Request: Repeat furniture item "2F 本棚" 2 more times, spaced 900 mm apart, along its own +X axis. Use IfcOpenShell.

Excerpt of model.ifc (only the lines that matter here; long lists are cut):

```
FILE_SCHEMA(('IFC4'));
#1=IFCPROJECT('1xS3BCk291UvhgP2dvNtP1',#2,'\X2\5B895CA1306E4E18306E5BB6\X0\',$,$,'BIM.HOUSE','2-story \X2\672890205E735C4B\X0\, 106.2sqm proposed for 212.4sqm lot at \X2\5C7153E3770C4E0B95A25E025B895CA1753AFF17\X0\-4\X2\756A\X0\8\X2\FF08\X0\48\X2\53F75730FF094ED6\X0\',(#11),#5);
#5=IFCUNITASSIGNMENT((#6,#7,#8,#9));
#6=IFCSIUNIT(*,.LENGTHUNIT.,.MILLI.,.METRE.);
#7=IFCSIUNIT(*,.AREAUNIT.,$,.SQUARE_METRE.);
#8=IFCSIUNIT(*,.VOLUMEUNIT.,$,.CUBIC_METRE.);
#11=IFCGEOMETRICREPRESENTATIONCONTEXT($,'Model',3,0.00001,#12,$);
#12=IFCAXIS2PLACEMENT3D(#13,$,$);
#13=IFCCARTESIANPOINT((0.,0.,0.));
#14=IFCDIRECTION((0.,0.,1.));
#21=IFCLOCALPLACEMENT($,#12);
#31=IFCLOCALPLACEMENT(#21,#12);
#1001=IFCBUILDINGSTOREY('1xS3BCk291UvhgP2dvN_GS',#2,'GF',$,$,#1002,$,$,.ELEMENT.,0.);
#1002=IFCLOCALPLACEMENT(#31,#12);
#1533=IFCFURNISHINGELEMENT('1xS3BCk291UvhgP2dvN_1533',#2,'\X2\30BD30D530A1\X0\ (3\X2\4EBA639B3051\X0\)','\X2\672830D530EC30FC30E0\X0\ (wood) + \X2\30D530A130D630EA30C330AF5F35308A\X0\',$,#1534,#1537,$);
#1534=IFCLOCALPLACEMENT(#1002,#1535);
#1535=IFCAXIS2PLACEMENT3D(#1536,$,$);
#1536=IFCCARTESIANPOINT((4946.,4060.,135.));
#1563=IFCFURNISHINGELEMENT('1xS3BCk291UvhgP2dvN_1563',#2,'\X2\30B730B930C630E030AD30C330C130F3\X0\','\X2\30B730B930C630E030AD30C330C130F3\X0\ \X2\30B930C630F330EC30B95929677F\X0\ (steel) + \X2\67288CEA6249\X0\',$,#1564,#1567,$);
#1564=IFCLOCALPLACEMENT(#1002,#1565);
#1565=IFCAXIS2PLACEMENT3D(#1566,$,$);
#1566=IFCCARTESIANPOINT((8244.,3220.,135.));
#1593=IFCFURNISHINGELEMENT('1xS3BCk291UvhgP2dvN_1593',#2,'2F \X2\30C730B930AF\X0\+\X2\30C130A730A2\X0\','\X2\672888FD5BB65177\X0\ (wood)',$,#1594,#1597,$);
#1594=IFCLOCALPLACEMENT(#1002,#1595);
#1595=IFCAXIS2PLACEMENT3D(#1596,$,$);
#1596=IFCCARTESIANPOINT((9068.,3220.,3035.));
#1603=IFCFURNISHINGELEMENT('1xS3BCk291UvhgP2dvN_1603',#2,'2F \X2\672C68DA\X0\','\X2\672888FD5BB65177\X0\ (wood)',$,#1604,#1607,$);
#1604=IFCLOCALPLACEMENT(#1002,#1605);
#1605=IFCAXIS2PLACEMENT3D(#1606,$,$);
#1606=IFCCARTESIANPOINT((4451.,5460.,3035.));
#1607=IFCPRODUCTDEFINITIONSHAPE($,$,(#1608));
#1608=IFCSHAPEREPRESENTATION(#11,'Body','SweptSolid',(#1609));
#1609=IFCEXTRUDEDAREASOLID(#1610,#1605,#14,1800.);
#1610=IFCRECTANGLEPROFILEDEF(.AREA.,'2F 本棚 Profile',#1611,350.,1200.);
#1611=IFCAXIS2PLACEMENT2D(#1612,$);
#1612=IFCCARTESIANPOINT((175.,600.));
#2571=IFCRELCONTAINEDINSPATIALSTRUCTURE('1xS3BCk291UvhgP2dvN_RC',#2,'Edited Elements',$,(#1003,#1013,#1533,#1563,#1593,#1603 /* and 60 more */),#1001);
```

```python
import ifcopenshell
import ifcopenshell.api.geometry
import ifcopenshell.api.root
import ifcopenshell.util.element
import ifcopenshell.util.placement
import ifcopenshell.util.unit

model = ifcopenshell.open("model.ifc")
unit_scale = ifcopenshell.util.unit.calculate_unit_scale(model)


def reuse_history(source, copy):
    """copy_class also copies each property set's owner history, people and application; keep the originals."""
    for rel in copy.IsDefinedBy:
        if rel.is_a("IfcRelDefinesByProperties") and (history := rel.RelatingPropertyDefinition.OwnerHistory):
            rel.RelatingPropertyDefinition.OwnerHistory = source.OwnerHistory
            ifcopenshell.util.element.remove_deep2(model, history)


source = model.by_guid("1xS3BCk291UvhgP2dvN_1603")
base = ifcopenshell.util.placement.get_local_placement(source.ObjectPlacement)
step = base[:3, 0] * 0.9 / unit_scale

for i in range(1, 3):
    copy = ifcopenshell.api.root.copy_class(model, product=source)
    copy.Representation = ifcopenshell.util.element.copy_deep(
        model, source.Representation, exclude=["IfcGeometricRepresentationContext", "IfcRepresentationMap"]
    )
    reuse_history(source, copy)
    matrix = base.copy()
    matrix[:3, 3] += i * step
    print("added at", matrix[:3, 3].round(3) + 0.0)
    ifcopenshell.api.geometry.edit_object_placement(model, product=copy, matrix=matrix, is_si=False)

model.write("model_updated.ifc")
```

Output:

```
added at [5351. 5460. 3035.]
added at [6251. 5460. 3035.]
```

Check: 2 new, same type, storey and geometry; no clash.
